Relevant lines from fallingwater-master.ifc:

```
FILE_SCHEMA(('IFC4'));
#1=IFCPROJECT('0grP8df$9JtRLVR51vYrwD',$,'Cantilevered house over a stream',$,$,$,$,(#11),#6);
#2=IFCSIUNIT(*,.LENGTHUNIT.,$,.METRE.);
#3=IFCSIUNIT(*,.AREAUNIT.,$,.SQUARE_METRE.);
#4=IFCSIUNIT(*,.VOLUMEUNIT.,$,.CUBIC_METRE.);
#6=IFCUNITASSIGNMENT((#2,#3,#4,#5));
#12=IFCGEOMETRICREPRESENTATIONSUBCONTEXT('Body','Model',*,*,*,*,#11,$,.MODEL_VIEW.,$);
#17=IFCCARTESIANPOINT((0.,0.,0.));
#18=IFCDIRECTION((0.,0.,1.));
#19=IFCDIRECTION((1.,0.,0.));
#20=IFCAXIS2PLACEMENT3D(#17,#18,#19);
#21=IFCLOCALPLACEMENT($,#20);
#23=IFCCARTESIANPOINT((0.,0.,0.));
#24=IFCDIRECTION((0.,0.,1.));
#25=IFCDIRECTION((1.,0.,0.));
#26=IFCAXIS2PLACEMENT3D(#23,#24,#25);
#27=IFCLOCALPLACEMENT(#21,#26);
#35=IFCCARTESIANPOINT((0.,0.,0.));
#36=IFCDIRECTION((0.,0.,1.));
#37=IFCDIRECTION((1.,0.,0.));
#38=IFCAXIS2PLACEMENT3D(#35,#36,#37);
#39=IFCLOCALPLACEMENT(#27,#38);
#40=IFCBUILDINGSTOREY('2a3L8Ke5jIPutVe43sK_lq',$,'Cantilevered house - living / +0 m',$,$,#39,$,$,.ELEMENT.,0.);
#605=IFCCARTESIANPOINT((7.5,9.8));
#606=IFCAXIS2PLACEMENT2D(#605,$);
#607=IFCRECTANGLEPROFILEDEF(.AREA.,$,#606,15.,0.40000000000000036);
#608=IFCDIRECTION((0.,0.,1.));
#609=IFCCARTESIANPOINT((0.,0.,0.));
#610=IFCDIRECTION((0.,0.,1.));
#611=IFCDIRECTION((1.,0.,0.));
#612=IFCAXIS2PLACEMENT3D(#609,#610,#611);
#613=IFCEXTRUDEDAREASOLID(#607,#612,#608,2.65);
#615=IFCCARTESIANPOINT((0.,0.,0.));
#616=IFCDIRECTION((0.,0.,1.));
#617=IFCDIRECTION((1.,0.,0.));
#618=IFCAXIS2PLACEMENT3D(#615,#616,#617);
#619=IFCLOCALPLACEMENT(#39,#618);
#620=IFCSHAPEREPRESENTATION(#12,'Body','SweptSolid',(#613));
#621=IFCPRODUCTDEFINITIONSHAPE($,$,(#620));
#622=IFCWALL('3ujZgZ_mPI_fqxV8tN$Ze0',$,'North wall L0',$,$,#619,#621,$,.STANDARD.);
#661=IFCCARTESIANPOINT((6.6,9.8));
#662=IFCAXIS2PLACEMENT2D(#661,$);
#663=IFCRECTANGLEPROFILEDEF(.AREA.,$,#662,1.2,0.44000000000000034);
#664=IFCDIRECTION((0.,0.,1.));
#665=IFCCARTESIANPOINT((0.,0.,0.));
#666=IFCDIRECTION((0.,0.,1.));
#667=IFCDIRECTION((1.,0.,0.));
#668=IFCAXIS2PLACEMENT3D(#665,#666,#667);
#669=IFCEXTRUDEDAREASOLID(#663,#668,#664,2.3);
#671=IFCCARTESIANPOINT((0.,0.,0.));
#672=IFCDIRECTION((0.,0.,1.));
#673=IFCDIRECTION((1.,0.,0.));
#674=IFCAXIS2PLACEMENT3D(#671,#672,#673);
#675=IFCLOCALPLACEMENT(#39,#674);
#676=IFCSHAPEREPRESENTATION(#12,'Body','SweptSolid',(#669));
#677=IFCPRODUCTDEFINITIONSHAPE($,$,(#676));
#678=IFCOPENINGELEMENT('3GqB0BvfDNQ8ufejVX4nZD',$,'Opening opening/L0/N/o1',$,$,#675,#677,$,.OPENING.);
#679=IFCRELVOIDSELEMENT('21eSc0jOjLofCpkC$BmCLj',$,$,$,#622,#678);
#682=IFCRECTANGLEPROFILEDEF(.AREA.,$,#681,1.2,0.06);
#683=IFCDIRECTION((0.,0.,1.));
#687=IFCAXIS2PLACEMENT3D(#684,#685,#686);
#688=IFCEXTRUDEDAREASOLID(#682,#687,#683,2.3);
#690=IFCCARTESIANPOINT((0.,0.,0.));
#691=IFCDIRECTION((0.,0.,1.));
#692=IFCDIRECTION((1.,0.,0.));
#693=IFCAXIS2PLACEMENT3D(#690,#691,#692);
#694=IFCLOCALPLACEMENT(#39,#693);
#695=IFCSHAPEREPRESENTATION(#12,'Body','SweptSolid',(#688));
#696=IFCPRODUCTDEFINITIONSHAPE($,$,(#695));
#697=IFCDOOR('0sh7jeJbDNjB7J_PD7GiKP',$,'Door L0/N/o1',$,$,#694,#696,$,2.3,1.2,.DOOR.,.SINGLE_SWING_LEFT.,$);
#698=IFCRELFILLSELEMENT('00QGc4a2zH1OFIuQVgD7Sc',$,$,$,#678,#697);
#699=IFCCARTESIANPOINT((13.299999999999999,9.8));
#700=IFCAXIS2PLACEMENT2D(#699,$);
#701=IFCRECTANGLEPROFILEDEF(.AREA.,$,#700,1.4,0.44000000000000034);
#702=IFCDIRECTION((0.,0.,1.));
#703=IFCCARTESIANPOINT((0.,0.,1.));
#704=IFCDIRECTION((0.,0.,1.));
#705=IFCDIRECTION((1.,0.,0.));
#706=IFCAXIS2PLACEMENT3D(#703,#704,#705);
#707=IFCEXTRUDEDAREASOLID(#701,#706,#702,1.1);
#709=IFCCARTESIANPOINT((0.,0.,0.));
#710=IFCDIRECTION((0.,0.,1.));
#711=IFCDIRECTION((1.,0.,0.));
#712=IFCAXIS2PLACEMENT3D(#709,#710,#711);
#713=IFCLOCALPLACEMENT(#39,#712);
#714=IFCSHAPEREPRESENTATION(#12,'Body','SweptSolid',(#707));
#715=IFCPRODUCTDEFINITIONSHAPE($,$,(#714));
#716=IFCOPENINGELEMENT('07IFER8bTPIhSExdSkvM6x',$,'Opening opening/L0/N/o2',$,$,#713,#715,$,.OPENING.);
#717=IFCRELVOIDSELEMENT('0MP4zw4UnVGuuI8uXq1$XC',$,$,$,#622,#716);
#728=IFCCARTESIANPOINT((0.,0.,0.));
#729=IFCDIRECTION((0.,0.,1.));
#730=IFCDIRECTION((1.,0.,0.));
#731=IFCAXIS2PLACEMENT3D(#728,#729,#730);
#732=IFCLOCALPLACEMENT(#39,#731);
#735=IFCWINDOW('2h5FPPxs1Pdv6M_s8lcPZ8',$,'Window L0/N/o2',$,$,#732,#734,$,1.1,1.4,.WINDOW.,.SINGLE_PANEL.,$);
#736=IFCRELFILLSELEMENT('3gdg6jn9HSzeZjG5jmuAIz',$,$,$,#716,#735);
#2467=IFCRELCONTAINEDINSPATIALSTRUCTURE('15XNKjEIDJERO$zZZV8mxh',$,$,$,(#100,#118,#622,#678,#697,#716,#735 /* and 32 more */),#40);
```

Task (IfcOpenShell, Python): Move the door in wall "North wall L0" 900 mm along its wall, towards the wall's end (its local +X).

```python
import ifcopenshell
import ifcopenshell.api.geometry
import ifcopenshell.util.placement
import ifcopenshell.util.unit

model = ifcopenshell.open("fallingwater-master.ifc")
unit_scale = ifcopenshell.util.unit.calculate_unit_scale(model)

door = model.by_guid("0sh7jeJbDNjB7J_PD7GiKP")
opening = door.FillsVoids[0].RelatingOpeningElement
wall = opening.VoidsElements[0].RelatingBuildingElement

wall_matrix = ifcopenshell.util.placement.get_local_placement(wall.ObjectPlacement)
shift = wall_matrix[:3, 0] * 0.9 / unit_scale
before = ifcopenshell.util.placement.get_local_placement(door.ObjectPlacement)[:3, 3].copy()

# The door is not placed relative to its opening, so move both.
for product in (opening, door):
    matrix = ifcopenshell.util.placement.get_local_placement(product.ObjectPlacement)
    matrix[:3, 3] += shift
    ifcopenshell.api.geometry.edit_object_placement(model, product=product, matrix=matrix, is_si=False)

after = ifcopenshell.util.placement.get_local_placement(door.ObjectPlacement)[:3, 3]
print("door moved by", (after - before).round(3) + 0.0)

model.write("fallingwater-master_rev.ifc")
```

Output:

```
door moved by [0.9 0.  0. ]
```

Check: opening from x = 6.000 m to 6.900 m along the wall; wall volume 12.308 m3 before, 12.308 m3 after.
